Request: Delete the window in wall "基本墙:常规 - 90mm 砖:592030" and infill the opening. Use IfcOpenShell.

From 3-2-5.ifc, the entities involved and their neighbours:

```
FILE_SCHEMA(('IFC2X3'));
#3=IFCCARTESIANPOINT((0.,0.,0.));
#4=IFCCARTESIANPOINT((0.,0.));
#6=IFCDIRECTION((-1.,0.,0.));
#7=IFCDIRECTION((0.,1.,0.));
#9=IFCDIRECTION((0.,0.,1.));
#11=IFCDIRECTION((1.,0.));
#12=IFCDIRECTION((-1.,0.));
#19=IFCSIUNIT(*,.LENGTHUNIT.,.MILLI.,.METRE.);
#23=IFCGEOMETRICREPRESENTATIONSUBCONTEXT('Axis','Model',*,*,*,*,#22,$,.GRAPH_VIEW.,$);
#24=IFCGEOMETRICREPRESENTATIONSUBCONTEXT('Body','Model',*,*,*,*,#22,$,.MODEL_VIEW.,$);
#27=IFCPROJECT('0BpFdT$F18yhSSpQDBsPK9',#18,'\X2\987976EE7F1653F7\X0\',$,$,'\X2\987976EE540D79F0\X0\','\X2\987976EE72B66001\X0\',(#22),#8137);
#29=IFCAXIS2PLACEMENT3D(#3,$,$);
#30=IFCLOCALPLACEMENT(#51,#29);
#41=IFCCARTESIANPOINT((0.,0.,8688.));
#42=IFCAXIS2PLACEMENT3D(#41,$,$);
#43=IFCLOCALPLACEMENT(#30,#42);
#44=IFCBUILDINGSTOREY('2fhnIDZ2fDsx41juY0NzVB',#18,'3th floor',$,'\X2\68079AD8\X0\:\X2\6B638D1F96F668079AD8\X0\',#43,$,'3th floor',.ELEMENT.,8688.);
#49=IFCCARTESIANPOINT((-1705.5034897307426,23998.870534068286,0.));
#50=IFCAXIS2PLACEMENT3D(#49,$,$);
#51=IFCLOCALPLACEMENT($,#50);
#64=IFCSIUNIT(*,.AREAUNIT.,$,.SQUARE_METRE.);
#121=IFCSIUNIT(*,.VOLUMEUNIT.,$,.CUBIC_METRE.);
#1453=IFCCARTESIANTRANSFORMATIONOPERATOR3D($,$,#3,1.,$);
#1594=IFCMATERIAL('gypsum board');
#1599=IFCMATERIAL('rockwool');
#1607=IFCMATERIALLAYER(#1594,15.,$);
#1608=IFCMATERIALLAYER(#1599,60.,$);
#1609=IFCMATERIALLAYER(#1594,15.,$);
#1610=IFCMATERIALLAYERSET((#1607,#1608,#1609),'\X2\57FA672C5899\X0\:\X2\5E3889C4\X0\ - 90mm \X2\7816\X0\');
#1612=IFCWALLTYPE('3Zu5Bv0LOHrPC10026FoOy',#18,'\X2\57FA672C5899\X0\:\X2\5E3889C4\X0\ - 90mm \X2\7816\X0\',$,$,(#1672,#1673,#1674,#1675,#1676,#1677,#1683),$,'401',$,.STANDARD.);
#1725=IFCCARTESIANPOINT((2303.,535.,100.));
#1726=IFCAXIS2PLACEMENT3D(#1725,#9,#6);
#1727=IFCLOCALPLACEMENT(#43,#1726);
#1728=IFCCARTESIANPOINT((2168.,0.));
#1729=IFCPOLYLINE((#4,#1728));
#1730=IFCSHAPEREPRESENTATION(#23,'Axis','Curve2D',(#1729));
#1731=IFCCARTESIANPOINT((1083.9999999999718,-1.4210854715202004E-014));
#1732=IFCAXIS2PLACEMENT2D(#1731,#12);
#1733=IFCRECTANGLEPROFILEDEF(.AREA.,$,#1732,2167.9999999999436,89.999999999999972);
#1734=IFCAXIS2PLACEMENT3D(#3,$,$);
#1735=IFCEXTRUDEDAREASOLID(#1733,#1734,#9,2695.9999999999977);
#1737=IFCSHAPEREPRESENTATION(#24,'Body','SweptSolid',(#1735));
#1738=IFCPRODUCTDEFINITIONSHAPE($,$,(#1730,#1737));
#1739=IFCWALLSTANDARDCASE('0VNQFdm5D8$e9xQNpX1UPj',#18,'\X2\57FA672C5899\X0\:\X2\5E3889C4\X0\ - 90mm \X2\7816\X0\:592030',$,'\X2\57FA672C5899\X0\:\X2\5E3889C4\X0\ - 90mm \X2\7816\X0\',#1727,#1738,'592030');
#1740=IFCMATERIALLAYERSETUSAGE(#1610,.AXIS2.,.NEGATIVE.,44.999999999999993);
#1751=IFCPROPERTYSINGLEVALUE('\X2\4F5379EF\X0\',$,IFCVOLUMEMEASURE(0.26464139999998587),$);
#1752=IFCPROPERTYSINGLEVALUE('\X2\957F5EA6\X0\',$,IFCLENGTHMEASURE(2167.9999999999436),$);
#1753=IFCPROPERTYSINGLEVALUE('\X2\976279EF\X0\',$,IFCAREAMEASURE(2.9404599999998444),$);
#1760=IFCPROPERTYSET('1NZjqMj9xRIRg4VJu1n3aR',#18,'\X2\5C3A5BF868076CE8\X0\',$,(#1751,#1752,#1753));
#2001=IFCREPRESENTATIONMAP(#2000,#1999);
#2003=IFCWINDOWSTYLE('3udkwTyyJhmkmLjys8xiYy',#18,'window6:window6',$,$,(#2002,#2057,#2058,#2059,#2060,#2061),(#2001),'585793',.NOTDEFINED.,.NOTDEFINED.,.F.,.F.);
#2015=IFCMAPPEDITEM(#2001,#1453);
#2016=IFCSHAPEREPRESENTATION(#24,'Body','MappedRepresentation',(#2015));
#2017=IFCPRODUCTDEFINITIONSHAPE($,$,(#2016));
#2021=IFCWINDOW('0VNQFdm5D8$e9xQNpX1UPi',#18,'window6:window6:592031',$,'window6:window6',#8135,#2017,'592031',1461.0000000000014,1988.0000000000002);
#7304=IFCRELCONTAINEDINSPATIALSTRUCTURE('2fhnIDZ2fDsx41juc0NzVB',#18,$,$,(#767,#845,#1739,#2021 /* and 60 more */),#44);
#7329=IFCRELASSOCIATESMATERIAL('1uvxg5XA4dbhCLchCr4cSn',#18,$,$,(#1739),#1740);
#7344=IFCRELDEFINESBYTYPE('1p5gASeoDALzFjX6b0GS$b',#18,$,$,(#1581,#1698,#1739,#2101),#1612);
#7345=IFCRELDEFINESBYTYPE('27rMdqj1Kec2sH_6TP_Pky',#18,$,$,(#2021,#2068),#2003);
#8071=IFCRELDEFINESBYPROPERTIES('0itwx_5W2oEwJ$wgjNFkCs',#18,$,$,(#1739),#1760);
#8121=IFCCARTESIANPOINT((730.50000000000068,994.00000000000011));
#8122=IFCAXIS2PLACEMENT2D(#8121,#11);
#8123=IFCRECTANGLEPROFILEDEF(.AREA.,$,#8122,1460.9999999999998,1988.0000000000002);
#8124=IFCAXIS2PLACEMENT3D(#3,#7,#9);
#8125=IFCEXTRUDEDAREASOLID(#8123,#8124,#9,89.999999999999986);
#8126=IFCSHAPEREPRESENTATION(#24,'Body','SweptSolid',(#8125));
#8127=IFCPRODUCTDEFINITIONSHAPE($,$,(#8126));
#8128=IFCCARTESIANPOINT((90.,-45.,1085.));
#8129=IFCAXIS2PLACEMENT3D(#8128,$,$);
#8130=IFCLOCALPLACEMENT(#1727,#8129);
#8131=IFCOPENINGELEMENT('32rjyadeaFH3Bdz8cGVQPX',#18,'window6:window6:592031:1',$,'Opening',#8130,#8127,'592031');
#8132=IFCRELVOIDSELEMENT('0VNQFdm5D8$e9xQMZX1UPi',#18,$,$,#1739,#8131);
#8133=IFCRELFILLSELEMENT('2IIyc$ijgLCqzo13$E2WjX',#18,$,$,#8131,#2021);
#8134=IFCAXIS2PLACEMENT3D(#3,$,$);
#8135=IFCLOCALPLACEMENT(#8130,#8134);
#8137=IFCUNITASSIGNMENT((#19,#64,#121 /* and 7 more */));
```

```python
import ifcopenshell
import ifcopenshell.api.feature
import ifcopenshell.api.pset
import ifcopenshell.api.root
import ifcopenshell.geom
import ifcopenshell.util.element
import ifcopenshell.util.shape
import ifcopenshell.util.unit

model = ifcopenshell.open("3-2-5.ifc")
area_scale = ifcopenshell.util.unit.calculate_unit_scale(model, "AREAUNIT")
volume_scale = ifcopenshell.util.unit.calculate_unit_scale(model, "VOLUMEUNIT")
settings = ifcopenshell.geom.settings()


def volume(element):
    """Net volume in cubic metres, openings subtracted."""
    shape = ifcopenshell.geom.create_shape(settings, element)
    return ifcopenshell.util.shape.get_volume(shape.geometry)


window = model.by_guid("0VNQFdm5D8$e9xQNpX1UPi")
opening = window.FillsVoids[0].RelatingOpeningElement
wall = opening.VoidsElements[0].RelatingBuildingElement
before = volume(wall)

ifcopenshell.api.root.remove_product(model, product=window)
ifcopenshell.api.feature.remove_feature(model, feature=opening)

after = volume(wall)
thickness = 0.09  # wall thickness in metres

# Update the wall's stored quantities.
pset = model.by_id(ifcopenshell.util.element.get_pset(wall, "尺寸标注", should_inherit=False)["id"])
ifcopenshell.api.pset.edit_pset(model, pset=pset, properties={
    "体积": model.create_entity("IfcVolumeMeasure", after / volume_scale),
    "面积": model.create_entity("IfcAreaMeasure", after / thickness / area_scale),
})

print(f"wall volume {before:.3f} -> {after:.3f} m3")

model.write("3-2-5-out.ifc")
```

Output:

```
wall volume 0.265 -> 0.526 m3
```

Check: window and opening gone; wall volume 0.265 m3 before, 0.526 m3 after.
